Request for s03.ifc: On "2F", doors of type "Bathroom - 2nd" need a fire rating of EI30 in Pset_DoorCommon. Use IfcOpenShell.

First a look at what the model holds.

```python
import ifcopenshell
import ifcopenshell.util.element

model = ifcopenshell.open("s03.ifc")
print(model.schema)
storey = next(s for s in model.by_type("IfcBuildingStorey") if s.Name == "2F")
doors = [e for e in ifcopenshell.util.element.get_decomposition(storey) if e.is_a("IfcDoor")]
seen = {}
for e in doors:
    element_type = ifcopenshell.util.element.get_type(e)
    key = (element_type.Name if element_type != e and element_type else None, ifcopenshell.util.element.get_pset(e, "Pset_DoorCommon", "FireRating"))
    seen[key] = seen.get(key, 0) + 1
for (name, value), count in sorted(seen.items(), key=str):
    print(count, "x", name, "|", value)
```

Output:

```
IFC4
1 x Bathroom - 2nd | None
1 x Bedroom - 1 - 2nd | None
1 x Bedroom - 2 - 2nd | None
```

```python
import ifcopenshell
import ifcopenshell.api.pset
import ifcopenshell.util.element

model = ifcopenshell.open("s03.ifc")

storey = next(s for s in model.by_type("IfcBuildingStorey") if s.Name == "2F")
doors = [e for e in ifcopenshell.util.element.get_decomposition(storey) if e.is_a("IfcDoor")]

count = 0
for e in doors:
    element_type = ifcopenshell.util.element.get_type(e)
    if element_type in (None, e) or element_type.Name != "Bathroom - 2nd":
        continue
    # add_pset returns the element's existing set when there is one.
    pset = ifcopenshell.api.pset.add_pset(model, product=e, name="Pset_DoorCommon")
    ifcopenshell.api.pset.edit_pset(model, pset=pset, properties={"FireRating": "EI30"})
    count += 1

print(count, "doors updated")

model.write("s03_v2.ifc")
```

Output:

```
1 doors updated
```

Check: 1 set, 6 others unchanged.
